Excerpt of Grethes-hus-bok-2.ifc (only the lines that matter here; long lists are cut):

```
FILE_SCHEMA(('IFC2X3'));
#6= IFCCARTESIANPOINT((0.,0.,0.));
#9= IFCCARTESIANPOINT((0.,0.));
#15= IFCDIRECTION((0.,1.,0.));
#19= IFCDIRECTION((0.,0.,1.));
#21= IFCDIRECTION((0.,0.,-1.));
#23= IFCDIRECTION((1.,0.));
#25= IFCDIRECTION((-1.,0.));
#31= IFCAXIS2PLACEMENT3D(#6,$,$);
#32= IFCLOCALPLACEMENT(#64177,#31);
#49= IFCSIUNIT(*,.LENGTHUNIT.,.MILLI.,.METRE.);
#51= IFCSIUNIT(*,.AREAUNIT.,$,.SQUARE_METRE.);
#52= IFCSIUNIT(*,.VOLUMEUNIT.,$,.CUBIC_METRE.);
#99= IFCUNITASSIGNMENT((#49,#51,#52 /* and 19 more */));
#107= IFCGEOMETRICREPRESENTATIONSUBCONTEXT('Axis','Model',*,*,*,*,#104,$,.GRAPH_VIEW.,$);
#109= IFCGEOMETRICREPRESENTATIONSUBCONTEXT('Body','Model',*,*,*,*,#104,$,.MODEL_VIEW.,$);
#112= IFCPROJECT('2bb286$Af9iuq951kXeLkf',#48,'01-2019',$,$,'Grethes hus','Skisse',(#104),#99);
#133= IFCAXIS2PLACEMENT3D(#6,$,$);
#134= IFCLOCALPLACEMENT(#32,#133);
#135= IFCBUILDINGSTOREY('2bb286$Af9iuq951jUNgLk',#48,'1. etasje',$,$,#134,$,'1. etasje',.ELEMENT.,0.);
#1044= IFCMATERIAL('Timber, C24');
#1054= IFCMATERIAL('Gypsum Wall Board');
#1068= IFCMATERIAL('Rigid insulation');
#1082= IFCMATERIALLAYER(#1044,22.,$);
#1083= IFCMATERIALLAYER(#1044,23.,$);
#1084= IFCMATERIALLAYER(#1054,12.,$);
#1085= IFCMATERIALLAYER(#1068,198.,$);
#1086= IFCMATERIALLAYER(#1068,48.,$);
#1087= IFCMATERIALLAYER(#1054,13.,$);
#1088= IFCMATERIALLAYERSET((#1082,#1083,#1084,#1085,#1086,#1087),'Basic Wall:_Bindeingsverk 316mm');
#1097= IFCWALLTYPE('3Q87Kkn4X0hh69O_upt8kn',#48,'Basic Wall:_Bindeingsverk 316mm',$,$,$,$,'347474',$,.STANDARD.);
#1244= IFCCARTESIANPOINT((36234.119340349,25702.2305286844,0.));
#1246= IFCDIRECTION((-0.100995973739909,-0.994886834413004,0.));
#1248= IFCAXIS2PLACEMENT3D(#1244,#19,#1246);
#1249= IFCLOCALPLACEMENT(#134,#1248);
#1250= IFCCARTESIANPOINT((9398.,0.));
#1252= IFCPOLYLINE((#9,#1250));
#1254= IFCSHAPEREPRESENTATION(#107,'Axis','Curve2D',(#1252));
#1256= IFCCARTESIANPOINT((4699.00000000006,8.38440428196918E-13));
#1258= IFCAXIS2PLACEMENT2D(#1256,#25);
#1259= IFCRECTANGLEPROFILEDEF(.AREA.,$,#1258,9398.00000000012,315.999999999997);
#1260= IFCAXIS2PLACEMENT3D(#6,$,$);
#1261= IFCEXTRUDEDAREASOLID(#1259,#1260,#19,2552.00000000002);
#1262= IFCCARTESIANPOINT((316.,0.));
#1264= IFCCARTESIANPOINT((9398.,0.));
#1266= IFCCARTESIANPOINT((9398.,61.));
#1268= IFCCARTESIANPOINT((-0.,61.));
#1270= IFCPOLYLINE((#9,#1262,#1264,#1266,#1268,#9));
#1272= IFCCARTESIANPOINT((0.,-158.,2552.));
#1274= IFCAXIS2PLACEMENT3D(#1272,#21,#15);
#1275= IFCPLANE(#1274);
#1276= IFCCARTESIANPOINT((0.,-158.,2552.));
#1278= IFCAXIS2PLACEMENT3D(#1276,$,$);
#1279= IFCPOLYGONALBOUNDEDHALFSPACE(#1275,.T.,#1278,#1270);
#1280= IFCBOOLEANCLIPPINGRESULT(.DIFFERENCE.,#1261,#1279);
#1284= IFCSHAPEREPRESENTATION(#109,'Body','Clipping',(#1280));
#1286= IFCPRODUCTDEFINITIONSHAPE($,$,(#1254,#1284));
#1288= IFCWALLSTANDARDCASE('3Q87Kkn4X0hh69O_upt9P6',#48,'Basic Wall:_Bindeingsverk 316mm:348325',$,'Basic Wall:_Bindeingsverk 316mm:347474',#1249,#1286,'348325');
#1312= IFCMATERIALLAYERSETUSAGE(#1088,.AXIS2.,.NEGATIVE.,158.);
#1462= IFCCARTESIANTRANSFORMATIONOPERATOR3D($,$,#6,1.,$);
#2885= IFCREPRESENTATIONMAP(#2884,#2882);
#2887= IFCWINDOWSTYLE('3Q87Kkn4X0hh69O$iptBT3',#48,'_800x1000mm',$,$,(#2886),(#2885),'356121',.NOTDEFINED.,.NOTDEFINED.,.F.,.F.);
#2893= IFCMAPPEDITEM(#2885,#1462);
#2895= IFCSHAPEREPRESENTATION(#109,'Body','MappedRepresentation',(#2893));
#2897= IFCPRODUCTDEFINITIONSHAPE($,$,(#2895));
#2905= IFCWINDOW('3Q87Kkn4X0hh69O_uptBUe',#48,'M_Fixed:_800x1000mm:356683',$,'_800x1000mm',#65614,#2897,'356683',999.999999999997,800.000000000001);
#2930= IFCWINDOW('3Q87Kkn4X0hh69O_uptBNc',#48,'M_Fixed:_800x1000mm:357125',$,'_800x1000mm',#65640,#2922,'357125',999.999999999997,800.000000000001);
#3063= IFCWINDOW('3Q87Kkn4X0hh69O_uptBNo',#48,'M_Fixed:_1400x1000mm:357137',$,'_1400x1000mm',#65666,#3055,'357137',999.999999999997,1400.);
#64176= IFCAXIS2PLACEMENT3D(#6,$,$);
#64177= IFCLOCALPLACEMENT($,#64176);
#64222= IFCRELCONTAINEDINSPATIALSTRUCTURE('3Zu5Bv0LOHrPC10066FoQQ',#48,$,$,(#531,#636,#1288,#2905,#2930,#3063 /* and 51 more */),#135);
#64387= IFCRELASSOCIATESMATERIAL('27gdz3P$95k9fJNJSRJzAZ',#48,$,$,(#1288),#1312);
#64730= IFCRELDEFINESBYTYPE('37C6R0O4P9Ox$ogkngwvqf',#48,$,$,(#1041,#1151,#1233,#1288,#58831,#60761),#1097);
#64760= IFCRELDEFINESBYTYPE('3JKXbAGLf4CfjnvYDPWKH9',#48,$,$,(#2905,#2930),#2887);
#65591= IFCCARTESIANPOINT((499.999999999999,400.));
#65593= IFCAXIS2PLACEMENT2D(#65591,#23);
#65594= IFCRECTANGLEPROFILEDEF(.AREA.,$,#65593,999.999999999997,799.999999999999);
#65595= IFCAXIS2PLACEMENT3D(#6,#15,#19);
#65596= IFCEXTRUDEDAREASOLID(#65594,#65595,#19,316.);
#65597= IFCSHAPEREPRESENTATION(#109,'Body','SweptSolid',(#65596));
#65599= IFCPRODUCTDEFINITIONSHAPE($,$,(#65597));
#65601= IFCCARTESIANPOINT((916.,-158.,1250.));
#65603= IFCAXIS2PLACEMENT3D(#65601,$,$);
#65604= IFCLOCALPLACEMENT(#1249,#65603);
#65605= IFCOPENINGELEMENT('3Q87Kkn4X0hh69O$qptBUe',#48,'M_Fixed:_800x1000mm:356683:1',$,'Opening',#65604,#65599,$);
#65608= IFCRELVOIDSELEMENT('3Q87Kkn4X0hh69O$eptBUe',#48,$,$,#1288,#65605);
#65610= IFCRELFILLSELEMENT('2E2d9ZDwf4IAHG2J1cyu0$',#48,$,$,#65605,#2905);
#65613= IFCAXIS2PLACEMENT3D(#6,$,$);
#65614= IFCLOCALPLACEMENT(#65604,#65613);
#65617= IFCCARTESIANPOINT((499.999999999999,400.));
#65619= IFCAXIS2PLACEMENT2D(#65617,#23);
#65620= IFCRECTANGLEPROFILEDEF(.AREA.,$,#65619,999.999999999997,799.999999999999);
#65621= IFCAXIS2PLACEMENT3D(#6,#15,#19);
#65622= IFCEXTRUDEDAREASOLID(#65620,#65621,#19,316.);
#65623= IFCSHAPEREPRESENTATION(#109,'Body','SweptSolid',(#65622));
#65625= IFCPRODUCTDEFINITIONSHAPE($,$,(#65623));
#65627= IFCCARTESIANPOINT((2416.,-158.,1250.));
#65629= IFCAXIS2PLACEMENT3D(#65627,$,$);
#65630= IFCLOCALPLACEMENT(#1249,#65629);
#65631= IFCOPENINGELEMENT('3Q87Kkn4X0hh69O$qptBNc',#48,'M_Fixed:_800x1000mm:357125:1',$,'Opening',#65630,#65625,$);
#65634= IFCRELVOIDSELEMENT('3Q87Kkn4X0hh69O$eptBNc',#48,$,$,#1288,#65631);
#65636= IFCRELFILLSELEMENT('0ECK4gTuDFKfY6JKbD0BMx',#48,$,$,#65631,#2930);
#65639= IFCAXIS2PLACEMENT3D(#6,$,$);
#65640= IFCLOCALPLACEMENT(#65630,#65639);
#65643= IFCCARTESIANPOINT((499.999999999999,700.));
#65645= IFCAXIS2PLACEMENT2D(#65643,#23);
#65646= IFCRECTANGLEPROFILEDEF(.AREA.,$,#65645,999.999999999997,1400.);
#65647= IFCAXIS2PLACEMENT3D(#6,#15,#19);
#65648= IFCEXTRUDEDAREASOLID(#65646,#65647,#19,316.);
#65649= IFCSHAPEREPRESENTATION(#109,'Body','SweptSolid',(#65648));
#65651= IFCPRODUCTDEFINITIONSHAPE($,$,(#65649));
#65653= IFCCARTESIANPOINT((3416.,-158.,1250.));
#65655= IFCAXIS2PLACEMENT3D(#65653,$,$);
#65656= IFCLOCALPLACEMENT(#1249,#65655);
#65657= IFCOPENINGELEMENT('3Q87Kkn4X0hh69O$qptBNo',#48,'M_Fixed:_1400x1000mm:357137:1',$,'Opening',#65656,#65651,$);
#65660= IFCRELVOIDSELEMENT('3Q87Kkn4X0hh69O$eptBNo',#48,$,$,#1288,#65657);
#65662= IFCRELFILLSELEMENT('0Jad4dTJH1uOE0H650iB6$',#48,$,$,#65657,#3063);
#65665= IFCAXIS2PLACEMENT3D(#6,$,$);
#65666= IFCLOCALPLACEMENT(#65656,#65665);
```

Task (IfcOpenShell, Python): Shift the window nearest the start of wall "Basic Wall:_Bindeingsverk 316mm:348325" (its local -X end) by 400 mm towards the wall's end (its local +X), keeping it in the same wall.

```python
import ifcopenshell
import ifcopenshell.api.geometry
import ifcopenshell.util.placement

model = ifcopenshell.open("Grethes-hus-bok-2.ifc")

window = model.by_guid("3Q87Kkn4X0hh69O_uptBUe")
opening = window.FillsVoids[0].RelatingOpeningElement
wall = opening.VoidsElements[0].RelatingBuildingElement

wall_matrix = ifcopenshell.util.placement.get_local_placement(wall.ObjectPlacement)
shift = wall_matrix[:3, 0] * 400.0
before = ifcopenshell.util.placement.get_local_placement(window.ObjectPlacement)[:3, 3].copy()

# The window is placed relative to its opening, so it follows when the opening moves.
matrix = ifcopenshell.util.placement.get_local_placement(opening.ObjectPlacement)
matrix[:3, 3] += shift
ifcopenshell.api.geometry.edit_object_placement(
    model, product=opening, matrix=matrix, is_si=False, should_transform_children=True
)

after = ifcopenshell.util.placement.get_local_placement(window.ObjectPlacement)[:3, 3]
print("window moved by", (after - before).round(3) + 0.0)

model.write("Grethes-hus-bok-2_updated.ifc")
```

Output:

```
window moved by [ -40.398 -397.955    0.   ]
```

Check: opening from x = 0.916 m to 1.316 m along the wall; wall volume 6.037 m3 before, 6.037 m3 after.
